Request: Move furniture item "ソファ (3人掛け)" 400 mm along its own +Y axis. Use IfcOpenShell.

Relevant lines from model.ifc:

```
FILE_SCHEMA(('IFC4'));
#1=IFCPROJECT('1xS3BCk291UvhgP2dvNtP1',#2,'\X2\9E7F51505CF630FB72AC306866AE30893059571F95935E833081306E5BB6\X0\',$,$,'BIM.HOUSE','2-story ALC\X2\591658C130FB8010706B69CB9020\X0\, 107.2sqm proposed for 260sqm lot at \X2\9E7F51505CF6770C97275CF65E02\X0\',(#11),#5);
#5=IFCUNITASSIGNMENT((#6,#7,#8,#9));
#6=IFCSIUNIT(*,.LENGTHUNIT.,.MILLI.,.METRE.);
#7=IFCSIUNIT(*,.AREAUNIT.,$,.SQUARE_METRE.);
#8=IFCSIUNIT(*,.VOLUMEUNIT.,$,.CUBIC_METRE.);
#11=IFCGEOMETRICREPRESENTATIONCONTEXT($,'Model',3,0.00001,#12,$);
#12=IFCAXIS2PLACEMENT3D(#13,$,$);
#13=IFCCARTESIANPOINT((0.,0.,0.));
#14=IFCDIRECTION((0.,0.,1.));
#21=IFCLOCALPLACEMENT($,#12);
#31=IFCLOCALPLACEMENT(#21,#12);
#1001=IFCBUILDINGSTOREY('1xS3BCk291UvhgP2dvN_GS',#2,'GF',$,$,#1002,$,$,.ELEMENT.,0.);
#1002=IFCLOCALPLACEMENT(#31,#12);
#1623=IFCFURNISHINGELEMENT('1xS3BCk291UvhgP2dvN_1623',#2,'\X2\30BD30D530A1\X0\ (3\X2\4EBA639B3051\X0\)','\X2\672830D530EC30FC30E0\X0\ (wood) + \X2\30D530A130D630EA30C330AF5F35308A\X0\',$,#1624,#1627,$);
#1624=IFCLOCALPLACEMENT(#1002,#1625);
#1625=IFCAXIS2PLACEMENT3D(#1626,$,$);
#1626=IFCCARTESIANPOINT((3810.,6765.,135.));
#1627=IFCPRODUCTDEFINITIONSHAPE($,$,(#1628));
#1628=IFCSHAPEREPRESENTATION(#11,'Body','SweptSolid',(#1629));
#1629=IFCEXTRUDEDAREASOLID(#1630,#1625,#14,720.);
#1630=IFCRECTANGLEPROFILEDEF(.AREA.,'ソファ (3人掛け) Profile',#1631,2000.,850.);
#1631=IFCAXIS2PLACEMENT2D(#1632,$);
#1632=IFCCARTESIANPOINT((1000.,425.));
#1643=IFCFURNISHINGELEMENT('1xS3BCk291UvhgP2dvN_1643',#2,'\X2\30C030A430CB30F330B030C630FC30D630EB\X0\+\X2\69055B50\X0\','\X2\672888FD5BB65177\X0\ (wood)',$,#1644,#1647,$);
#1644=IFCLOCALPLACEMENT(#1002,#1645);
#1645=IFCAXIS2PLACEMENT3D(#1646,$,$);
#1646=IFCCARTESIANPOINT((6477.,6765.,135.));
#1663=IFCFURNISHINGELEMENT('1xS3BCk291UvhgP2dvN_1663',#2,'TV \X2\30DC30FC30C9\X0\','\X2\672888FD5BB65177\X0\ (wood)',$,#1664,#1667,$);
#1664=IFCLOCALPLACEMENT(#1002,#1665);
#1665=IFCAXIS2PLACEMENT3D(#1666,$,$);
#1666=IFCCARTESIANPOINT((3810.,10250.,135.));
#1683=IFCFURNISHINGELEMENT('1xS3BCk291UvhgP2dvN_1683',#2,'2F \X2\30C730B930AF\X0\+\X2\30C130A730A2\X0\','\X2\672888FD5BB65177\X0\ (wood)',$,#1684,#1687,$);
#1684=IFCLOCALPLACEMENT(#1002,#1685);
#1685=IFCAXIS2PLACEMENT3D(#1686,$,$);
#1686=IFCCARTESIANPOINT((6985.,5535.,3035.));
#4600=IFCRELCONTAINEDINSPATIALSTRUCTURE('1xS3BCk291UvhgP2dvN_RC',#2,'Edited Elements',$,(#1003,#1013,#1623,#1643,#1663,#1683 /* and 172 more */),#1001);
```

```python
import ifcopenshell
import ifcopenshell.api.geometry
import ifcopenshell.util.placement
import ifcopenshell.util.unit

model = ifcopenshell.open("model.ifc")
unit_scale = ifcopenshell.util.unit.calculate_unit_scale(model)

item = model.by_id(1623)
matrix = ifcopenshell.util.placement.get_local_placement(item.ObjectPlacement)
matrix[:3, 3] += matrix[:3, 1] * 0.4 / unit_scale
ifcopenshell.api.geometry.edit_object_placement(model, product=item, matrix=matrix, is_si=False)

print(ifcopenshell.util.placement.get_local_placement(item.ObjectPlacement).round(3) + 0.0)

model.write("model_rev.ifc")
```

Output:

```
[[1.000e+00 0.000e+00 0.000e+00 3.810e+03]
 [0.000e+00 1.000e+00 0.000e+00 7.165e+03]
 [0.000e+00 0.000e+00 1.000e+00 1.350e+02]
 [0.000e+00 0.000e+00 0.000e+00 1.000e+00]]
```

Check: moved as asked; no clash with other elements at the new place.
